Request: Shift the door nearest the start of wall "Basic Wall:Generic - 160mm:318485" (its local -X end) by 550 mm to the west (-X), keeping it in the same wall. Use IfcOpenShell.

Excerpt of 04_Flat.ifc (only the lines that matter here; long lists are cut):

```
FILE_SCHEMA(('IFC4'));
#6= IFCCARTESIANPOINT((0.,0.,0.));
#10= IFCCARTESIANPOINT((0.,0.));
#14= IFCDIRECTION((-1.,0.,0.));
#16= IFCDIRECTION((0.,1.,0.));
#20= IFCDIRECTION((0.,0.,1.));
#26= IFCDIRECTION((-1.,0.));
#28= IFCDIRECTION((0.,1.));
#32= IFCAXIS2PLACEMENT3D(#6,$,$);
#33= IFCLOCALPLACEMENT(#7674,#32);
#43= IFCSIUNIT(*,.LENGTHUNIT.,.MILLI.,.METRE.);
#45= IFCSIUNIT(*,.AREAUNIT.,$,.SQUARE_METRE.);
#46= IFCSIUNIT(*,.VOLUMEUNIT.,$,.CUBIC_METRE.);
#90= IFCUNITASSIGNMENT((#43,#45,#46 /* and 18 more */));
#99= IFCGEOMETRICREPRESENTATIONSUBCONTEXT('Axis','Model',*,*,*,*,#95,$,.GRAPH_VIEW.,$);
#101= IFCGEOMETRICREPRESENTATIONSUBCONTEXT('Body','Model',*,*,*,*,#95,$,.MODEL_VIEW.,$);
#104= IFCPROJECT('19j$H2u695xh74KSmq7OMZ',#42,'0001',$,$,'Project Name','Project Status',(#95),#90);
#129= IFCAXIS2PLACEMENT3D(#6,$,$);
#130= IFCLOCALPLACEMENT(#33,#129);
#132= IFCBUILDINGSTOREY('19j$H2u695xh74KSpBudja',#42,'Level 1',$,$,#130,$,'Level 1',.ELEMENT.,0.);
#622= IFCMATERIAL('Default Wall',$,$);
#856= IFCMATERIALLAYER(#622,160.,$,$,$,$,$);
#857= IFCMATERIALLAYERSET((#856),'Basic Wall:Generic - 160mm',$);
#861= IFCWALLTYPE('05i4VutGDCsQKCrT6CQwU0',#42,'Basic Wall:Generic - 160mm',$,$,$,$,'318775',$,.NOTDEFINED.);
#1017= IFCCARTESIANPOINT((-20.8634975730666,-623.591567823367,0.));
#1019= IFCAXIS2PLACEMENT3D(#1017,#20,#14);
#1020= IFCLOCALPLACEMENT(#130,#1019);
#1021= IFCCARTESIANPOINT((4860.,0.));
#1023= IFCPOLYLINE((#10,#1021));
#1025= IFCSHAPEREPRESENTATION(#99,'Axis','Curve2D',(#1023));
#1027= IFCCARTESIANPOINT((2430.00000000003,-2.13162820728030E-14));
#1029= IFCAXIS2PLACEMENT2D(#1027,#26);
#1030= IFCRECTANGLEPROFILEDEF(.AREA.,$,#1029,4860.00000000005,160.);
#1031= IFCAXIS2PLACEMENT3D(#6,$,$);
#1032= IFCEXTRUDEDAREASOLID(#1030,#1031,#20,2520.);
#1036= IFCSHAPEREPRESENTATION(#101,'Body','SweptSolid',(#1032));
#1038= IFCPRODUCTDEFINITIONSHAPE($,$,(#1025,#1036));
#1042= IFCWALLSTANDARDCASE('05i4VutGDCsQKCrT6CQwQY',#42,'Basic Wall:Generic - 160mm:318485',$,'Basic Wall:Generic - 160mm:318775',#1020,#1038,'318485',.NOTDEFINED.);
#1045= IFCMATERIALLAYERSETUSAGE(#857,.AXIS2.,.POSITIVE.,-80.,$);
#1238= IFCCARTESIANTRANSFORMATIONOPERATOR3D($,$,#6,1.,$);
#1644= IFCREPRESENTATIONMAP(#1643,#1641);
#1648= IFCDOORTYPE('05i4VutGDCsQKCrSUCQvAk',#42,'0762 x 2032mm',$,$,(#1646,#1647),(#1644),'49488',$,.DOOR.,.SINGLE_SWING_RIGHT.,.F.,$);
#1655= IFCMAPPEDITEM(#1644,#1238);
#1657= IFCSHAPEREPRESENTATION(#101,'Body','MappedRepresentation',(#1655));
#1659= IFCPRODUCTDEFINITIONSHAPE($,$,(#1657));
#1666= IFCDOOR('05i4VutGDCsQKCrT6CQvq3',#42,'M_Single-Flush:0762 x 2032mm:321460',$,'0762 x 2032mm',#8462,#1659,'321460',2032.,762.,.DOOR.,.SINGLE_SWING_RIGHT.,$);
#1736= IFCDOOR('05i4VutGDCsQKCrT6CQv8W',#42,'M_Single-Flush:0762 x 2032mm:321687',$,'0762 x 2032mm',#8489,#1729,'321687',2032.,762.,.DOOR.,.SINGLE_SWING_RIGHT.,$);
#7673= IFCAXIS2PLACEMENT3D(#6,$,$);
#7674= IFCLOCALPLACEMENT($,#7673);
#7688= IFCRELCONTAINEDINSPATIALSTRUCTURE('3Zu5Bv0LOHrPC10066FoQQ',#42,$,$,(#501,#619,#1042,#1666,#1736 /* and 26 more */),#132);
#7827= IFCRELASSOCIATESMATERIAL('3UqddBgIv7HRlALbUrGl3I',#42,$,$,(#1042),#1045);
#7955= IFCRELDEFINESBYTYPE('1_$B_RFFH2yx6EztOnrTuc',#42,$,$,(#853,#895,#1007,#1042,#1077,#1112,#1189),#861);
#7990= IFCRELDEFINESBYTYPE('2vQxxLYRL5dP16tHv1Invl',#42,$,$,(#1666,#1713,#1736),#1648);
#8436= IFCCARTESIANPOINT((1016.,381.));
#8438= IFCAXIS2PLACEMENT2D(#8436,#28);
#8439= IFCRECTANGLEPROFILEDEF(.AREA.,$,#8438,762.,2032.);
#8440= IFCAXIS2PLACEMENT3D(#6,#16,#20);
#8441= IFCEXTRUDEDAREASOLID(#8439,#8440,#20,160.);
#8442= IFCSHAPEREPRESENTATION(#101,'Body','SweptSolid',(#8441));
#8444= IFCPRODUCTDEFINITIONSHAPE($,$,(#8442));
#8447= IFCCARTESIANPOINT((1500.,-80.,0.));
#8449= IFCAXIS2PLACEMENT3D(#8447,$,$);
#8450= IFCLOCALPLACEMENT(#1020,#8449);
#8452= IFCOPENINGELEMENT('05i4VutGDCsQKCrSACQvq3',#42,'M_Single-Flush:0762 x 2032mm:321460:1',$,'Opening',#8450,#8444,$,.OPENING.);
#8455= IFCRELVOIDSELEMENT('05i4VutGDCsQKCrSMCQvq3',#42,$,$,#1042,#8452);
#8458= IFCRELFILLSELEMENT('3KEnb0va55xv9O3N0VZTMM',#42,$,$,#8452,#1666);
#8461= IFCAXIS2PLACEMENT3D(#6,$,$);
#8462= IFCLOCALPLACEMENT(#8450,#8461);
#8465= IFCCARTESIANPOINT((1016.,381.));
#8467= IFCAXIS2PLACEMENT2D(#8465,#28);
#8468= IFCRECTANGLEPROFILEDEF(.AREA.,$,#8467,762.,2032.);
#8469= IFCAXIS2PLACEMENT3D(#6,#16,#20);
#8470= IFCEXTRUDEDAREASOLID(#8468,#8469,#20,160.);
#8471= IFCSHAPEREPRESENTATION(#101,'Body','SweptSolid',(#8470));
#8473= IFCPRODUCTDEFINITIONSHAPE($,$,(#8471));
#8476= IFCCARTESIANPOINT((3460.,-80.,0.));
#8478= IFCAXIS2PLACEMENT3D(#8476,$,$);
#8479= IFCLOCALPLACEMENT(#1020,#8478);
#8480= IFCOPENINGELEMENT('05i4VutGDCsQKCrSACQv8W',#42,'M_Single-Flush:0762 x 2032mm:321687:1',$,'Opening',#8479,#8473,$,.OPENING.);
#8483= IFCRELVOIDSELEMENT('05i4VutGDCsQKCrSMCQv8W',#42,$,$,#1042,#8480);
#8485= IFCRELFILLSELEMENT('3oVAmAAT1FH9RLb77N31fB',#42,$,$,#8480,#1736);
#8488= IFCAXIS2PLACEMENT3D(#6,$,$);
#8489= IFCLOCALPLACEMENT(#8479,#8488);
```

```python
import ifcopenshell
import ifcopenshell.api.geometry
import ifcopenshell.util.placement
import ifcopenshell.util.unit

model = ifcopenshell.open("04_Flat.ifc")
unit_scale = ifcopenshell.util.unit.calculate_unit_scale(model)

door = model.by_guid("05i4VutGDCsQKCrT6CQvq3")
opening = door.FillsVoids[0].RelatingOpeningElement
wall = opening.VoidsElements[0].RelatingBuildingElement

wall_matrix = ifcopenshell.util.placement.get_local_placement(wall.ObjectPlacement)
shift = wall_matrix[:3, 0] * 0.55 / unit_scale
before = ifcopenshell.util.placement.get_local_placement(door.ObjectPlacement)[:3, 3].copy()

# The door is placed relative to its opening, so it follows when the opening moves.
matrix = ifcopenshell.util.placement.get_local_placement(opening.ObjectPlacement)
matrix[:3, 3] += shift
ifcopenshell.api.geometry.edit_object_placement(
    model, product=opening, matrix=matrix, is_si=False, should_transform_children=True
)

after = ifcopenshell.util.placement.get_local_placement(door.ObjectPlacement)[:3, 3]
print("door moved by", (after - before).round(3) + 0.0)

model.write("04_Flat_rev.ifc")
```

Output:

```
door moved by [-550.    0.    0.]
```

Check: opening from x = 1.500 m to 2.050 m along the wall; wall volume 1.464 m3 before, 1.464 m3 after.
